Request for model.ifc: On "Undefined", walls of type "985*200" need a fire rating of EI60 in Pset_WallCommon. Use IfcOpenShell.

First a look at what the model holds.

```python
import ifcopenshell
import ifcopenshell.util.element

model = ifcopenshell.open("model.ifc")
print(model.schema)
storey = next(s for s in model.by_type("IfcBuildingStorey") if s.Name == "Undefined")
walls = [e for e in ifcopenshell.util.element.get_decomposition(storey) if e.is_a("IfcWall")]
seen = {}
for e in walls:
    element_type = ifcopenshell.util.element.get_type(e)
    key = (element_type.Name if element_type != e and element_type else None, ifcopenshell.util.element.get_pset(e, "Pset_WallCommon", "FireRating"))
    seen[key] = seen.get(key, 0) + 1
for (name, value), count in sorted(seen.items(), key=str):
    print(count, "x", name, "|", value)
```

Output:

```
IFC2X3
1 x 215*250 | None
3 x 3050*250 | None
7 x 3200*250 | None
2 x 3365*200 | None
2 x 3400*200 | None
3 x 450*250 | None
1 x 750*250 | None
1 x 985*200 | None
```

```python
import ifcopenshell
import ifcopenshell.api.pset
import ifcopenshell.util.element

model = ifcopenshell.open("model.ifc")

storey = next(s for s in model.by_type("IfcBuildingStorey") if s.Name == "Undefined")
walls = [e for e in ifcopenshell.util.element.get_decomposition(storey) if e.is_a("IfcWall")]

count = 0
for e in walls:
    element_type = ifcopenshell.util.element.get_type(e)
    if element_type in (None, e) or element_type.Name != "985*200":
        continue
    # add_pset returns the element's existing set when there is one.
    pset = ifcopenshell.api.pset.add_pset(model, product=e, name="Pset_WallCommon")
    ifcopenshell.api.pset.edit_pset(model, pset=pset, properties={"FireRating": "EI60"})
    count += 1

print(count, "walls updated")

model.write("model_rev.ifc")
```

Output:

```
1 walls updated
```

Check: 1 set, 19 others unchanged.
